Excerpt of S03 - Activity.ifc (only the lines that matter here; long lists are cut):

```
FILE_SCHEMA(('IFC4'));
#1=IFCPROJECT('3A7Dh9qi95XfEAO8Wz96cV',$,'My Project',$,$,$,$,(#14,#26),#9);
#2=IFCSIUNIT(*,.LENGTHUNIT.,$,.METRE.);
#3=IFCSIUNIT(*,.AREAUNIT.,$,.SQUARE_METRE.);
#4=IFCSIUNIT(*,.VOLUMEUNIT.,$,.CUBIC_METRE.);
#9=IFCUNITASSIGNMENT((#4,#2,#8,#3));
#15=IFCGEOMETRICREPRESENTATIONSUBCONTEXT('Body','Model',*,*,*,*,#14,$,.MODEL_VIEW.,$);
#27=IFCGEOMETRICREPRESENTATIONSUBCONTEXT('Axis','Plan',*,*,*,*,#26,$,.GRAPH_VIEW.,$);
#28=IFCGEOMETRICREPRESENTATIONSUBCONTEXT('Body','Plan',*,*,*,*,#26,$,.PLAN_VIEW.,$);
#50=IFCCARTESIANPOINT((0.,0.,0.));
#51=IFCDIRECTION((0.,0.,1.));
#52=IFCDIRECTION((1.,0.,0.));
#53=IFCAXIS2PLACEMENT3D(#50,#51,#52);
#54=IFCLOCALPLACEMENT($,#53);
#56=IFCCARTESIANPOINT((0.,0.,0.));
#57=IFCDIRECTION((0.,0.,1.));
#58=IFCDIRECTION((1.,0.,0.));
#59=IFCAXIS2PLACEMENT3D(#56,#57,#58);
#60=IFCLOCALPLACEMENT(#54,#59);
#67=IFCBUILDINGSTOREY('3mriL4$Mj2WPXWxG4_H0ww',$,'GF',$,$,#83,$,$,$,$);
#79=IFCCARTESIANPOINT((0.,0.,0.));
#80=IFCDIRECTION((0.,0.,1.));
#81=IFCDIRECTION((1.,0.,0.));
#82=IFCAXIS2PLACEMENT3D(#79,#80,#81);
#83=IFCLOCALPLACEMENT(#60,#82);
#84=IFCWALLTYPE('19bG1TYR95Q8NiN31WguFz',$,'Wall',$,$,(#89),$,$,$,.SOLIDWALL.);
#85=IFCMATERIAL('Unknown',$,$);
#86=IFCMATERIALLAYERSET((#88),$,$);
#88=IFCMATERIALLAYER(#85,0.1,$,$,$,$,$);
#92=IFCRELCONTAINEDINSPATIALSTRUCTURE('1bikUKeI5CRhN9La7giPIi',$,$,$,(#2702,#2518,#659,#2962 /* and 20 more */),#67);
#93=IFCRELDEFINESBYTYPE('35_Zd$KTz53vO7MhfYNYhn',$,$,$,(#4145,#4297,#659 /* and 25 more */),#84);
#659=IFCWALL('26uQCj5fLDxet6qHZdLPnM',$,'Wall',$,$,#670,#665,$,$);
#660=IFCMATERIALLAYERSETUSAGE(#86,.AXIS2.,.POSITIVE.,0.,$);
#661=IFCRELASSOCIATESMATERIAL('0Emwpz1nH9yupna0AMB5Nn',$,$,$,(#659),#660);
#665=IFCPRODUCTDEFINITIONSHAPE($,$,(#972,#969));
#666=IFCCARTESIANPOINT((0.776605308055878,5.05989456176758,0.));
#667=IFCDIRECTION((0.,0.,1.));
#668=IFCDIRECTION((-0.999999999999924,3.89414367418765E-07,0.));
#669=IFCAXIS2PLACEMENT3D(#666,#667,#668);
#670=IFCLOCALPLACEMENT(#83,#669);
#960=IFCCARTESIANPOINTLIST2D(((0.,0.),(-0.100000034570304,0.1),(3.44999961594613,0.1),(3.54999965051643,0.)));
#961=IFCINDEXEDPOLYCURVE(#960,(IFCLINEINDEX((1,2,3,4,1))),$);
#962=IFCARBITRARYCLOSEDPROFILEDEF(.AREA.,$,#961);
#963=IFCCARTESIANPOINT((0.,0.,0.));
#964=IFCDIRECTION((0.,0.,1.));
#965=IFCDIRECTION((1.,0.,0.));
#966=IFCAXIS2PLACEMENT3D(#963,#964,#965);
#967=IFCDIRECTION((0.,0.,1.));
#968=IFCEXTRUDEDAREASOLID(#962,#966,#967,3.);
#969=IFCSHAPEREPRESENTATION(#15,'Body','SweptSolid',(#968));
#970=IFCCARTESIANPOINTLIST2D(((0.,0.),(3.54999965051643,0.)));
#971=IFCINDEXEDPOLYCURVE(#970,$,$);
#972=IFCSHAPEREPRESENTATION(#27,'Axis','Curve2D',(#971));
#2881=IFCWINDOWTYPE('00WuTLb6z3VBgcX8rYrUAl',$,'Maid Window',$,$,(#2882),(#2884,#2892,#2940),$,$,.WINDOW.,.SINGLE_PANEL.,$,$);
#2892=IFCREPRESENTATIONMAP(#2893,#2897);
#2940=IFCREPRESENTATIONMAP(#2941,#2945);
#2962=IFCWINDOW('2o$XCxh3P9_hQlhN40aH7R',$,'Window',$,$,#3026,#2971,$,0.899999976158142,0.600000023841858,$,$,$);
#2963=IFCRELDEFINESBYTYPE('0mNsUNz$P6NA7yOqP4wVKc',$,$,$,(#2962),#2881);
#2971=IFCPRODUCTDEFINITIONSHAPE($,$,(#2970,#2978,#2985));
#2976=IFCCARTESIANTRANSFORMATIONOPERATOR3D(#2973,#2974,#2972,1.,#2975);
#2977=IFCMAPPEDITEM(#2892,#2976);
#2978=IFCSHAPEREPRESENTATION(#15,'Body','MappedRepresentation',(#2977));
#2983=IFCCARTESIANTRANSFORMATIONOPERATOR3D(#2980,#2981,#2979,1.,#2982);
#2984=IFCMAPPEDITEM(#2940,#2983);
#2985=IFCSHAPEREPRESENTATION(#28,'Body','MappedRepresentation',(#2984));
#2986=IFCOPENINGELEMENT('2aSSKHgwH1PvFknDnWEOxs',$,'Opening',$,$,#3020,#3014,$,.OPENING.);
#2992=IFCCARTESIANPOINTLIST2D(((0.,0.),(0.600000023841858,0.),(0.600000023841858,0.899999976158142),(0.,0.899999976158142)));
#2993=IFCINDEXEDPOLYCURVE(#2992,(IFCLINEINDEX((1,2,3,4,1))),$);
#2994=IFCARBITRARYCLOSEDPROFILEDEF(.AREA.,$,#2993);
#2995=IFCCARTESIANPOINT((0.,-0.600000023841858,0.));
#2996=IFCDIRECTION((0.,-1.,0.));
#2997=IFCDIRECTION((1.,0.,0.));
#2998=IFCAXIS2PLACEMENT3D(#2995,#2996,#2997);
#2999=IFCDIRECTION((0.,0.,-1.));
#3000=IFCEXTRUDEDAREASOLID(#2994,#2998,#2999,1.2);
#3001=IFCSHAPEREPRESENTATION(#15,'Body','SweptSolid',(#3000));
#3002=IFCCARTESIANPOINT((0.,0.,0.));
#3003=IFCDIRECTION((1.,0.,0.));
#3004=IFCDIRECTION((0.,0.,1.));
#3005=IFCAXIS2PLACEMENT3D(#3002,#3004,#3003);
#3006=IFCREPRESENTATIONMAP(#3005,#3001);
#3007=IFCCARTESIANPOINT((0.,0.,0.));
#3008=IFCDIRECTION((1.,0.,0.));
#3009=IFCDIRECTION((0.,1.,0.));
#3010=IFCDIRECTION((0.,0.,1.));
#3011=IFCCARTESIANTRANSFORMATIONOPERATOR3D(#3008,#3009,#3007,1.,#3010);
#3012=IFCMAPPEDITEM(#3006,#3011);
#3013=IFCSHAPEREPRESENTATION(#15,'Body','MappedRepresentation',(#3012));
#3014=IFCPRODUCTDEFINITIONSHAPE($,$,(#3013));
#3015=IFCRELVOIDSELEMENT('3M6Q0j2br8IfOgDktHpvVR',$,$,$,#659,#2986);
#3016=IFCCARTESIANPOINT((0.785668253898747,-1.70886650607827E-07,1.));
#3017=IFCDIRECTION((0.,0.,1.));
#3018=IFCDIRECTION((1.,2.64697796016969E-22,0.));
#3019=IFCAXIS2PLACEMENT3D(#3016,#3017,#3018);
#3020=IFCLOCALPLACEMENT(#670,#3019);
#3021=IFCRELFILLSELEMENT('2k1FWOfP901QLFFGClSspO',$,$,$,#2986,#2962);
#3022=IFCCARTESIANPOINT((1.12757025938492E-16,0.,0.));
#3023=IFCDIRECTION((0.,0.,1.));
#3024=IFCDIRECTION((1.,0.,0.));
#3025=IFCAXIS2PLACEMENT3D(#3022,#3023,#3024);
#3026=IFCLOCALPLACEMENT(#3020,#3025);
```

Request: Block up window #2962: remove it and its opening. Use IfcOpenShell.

```python
import ifcopenshell
import ifcopenshell.api.feature
import ifcopenshell.api.root
import ifcopenshell.geom
import ifcopenshell.util.shape

model = ifcopenshell.open("S03 - Activity.ifc")
settings = ifcopenshell.geom.settings()


def volume(element):
    """Net volume in cubic metres, openings subtracted."""
    shape = ifcopenshell.geom.create_shape(settings, element)
    return ifcopenshell.util.shape.get_volume(shape.geometry)


window = model.by_id(2962)
opening = window.FillsVoids[0].RelatingOpeningElement
wall = opening.VoidsElements[0].RelatingBuildingElement
before = volume(wall)

ifcopenshell.api.root.remove_product(model, product=window)
ifcopenshell.api.feature.remove_feature(model, feature=opening)

after = volume(wall)

print(f"wall volume {before:.3f} -> {after:.3f} m3")

model.write("S03 - Activity_rev.ifc")
```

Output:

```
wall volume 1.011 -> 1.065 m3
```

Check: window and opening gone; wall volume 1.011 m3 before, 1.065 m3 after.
